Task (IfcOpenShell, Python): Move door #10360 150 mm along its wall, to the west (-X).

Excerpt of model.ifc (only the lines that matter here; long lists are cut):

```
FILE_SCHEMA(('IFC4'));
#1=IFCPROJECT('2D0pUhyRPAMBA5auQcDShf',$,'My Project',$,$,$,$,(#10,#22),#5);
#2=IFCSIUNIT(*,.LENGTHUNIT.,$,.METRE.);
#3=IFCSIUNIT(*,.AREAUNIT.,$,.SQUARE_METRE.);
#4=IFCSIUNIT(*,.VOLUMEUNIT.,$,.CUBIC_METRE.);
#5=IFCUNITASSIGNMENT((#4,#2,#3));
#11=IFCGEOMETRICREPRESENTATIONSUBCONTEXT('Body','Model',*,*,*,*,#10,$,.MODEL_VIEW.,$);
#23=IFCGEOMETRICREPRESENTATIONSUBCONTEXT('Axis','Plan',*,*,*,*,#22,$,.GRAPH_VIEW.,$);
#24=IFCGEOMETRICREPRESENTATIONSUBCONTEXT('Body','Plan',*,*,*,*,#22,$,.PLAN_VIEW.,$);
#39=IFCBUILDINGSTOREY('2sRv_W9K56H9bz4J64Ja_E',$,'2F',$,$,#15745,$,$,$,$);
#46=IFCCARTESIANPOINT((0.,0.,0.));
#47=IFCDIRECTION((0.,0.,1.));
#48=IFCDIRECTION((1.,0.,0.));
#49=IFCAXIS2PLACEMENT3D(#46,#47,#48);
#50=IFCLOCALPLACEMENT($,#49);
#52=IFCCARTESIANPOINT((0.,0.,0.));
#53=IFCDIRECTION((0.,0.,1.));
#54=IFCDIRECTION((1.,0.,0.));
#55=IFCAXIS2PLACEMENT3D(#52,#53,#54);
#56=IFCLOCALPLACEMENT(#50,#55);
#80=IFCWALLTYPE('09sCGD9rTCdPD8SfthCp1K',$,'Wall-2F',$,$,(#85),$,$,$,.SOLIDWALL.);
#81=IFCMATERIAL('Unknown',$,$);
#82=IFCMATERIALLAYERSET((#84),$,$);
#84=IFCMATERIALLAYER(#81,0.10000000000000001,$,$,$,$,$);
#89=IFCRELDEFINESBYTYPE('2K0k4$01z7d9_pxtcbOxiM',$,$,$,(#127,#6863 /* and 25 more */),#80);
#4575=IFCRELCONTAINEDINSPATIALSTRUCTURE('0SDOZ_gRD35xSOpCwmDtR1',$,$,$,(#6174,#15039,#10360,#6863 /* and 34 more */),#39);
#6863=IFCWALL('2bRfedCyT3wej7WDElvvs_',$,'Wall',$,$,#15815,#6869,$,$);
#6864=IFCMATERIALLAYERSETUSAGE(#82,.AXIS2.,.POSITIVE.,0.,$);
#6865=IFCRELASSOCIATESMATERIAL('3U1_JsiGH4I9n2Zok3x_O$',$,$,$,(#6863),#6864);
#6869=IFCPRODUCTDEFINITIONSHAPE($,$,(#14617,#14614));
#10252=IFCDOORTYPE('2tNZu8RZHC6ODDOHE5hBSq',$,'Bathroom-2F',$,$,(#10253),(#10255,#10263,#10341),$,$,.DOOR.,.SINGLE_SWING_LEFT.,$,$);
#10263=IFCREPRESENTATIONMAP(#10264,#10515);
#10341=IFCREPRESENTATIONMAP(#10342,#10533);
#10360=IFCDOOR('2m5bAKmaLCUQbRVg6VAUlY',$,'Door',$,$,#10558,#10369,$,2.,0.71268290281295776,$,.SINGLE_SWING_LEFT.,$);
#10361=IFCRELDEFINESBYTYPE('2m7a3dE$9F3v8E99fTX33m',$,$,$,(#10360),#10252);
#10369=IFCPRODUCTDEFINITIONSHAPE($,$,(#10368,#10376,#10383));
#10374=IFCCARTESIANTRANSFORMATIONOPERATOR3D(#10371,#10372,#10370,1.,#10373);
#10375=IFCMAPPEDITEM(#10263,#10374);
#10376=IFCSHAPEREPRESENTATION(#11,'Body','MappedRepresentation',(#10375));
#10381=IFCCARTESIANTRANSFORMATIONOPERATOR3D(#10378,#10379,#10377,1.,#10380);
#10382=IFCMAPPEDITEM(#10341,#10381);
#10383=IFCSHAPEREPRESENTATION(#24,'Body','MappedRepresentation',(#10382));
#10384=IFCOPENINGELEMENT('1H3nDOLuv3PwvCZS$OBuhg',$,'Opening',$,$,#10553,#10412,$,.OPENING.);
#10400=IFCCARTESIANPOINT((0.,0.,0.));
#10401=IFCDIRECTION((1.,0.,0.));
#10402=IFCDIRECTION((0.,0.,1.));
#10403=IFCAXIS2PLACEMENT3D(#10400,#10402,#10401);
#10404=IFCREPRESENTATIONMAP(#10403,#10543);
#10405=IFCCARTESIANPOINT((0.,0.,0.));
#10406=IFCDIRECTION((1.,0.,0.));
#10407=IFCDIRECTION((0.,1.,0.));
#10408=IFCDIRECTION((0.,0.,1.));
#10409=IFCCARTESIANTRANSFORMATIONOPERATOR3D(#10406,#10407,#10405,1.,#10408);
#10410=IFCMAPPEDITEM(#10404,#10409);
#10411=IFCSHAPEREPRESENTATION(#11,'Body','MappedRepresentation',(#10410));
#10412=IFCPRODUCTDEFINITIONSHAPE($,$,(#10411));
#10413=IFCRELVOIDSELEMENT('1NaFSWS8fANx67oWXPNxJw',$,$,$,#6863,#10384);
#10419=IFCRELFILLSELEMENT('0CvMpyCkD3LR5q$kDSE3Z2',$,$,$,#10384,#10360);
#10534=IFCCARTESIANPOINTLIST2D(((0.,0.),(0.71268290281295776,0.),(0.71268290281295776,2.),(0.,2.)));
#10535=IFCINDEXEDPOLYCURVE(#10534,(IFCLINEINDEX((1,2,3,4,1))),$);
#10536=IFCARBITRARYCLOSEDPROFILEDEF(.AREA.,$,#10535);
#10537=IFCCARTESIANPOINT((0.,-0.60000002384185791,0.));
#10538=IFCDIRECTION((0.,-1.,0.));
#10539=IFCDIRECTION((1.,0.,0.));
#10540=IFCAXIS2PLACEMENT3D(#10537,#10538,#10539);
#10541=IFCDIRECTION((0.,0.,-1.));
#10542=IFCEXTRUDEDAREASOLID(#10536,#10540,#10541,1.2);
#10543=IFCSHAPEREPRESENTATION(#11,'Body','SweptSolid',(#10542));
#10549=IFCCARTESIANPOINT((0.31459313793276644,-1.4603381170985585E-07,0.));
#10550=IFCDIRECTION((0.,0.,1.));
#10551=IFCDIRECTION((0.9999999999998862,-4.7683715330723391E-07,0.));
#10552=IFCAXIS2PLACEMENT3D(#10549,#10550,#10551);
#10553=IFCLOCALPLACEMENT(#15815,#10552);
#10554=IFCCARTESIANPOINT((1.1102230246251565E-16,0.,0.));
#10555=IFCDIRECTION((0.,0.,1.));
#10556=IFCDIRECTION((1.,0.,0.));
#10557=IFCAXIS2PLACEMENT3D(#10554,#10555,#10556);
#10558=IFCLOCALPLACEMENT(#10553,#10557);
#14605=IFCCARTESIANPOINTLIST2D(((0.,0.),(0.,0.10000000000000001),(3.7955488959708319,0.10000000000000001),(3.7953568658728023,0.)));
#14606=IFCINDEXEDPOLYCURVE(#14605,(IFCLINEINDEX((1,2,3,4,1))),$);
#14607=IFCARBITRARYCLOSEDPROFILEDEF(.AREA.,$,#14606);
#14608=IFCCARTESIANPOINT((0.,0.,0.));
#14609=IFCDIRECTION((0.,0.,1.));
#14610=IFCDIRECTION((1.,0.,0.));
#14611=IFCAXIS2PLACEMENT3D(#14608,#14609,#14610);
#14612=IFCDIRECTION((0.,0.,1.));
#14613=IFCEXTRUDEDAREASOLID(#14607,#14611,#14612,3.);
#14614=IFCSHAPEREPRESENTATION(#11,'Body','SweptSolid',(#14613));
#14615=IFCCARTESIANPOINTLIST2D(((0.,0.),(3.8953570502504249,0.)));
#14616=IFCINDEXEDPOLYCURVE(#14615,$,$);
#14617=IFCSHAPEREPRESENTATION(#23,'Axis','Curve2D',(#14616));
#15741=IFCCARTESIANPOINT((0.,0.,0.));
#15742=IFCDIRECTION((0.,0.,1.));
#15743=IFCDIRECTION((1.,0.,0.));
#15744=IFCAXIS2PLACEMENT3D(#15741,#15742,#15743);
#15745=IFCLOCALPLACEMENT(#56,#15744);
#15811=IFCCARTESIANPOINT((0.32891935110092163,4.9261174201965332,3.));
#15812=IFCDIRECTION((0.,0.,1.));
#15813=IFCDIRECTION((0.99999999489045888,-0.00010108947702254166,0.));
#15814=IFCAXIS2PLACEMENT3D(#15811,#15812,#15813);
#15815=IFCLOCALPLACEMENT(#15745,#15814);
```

```python
import ifcopenshell
import ifcopenshell.api.geometry
import ifcopenshell.util.placement
import ifcopenshell.util.unit

model = ifcopenshell.open("model.ifc")
unit_scale = ifcopenshell.util.unit.calculate_unit_scale(model)

door = model.by_id(10360)
opening = door.FillsVoids[0].RelatingOpeningElement
wall = opening.VoidsElements[0].RelatingBuildingElement

wall_matrix = ifcopenshell.util.placement.get_local_placement(wall.ObjectPlacement)
shift = wall_matrix[:3, 0] * -0.15 / unit_scale
before = ifcopenshell.util.placement.get_local_placement(door.ObjectPlacement)[:3, 3].copy()

# The door is placed relative to its opening, so it follows when the opening moves.
matrix = ifcopenshell.util.placement.get_local_placement(opening.ObjectPlacement)
matrix[:3, 3] += shift
ifcopenshell.api.geometry.edit_object_placement(
    model, product=opening, matrix=matrix, is_si=False, should_transform_children=True
)

after = ifcopenshell.util.placement.get_local_placement(door.ObjectPlacement)[:3, 3]
print("door moved by", (after - before).round(3) + 0.0)

model.write("model_updated.ifc")
```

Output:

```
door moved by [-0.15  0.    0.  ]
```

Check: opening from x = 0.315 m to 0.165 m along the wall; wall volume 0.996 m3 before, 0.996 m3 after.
